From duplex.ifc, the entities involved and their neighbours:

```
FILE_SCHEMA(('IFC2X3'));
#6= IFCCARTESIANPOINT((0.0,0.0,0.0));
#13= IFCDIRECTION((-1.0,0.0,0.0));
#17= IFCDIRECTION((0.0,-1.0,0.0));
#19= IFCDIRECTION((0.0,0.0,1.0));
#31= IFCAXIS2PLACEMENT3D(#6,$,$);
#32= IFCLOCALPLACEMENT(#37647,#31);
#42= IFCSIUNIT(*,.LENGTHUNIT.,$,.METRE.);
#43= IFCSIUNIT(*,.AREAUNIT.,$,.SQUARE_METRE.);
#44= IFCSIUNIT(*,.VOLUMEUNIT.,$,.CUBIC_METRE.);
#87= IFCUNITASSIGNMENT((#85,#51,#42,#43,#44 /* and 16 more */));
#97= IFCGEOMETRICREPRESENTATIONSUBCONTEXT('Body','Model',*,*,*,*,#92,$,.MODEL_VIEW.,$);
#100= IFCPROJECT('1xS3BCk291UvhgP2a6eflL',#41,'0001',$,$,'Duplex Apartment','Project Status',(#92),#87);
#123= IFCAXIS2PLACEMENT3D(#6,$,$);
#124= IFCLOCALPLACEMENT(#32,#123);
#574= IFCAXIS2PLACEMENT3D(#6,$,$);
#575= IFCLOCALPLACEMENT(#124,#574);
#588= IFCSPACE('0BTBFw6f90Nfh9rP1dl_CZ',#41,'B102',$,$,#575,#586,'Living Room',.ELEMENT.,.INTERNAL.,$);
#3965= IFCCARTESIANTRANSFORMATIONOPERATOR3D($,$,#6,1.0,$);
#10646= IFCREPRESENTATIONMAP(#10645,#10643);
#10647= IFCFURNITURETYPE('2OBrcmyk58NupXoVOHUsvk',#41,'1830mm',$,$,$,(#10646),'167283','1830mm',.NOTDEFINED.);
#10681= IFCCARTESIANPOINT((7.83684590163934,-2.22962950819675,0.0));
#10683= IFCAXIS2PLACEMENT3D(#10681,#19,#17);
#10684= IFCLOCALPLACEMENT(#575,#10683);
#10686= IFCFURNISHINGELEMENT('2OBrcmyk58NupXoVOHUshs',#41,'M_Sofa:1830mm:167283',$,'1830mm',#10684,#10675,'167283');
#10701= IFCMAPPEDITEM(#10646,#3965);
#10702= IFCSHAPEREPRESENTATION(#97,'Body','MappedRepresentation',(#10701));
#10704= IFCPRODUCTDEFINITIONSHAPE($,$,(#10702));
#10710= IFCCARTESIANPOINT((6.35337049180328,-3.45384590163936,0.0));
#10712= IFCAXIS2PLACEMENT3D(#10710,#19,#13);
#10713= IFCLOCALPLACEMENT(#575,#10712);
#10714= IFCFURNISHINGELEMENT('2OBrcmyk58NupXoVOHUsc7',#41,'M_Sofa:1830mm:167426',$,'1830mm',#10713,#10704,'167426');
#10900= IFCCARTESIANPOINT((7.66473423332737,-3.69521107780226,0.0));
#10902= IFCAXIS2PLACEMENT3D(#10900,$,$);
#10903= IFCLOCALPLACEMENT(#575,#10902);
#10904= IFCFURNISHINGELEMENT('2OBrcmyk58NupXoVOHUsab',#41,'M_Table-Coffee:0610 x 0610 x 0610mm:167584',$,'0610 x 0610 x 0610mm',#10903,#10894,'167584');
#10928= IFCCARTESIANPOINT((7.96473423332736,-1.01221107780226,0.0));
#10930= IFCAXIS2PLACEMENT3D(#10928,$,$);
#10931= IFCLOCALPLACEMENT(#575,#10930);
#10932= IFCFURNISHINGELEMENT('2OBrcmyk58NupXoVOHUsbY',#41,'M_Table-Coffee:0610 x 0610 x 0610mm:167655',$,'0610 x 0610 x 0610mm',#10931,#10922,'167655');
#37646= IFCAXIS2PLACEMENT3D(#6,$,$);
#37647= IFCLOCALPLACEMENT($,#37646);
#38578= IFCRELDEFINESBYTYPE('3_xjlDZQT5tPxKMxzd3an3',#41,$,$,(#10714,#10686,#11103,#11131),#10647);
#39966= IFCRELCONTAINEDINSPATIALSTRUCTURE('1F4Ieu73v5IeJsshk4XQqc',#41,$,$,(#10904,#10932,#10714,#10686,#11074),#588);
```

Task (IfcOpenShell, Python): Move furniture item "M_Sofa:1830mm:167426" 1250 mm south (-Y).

```python
import ifcopenshell
import ifcopenshell.api.geometry
import ifcopenshell.util.placement
import ifcopenshell.util.unit

model = ifcopenshell.open("duplex.ifc")
unit_scale = ifcopenshell.util.unit.calculate_unit_scale(model)

item = model.by_guid("2OBrcmyk58NupXoVOHUsc7")
matrix = ifcopenshell.util.placement.get_local_placement(item.ObjectPlacement)
matrix[1, 3] -= 1.25 / unit_scale
ifcopenshell.api.geometry.edit_object_placement(model, product=item, matrix=matrix, is_si=False)

print(ifcopenshell.util.placement.get_local_placement(item.ObjectPlacement).round(3) + 0.0)

model.write("duplex-out.ifc")
```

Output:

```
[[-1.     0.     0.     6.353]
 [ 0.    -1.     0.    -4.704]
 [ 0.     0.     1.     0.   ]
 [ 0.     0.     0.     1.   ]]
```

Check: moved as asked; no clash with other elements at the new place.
